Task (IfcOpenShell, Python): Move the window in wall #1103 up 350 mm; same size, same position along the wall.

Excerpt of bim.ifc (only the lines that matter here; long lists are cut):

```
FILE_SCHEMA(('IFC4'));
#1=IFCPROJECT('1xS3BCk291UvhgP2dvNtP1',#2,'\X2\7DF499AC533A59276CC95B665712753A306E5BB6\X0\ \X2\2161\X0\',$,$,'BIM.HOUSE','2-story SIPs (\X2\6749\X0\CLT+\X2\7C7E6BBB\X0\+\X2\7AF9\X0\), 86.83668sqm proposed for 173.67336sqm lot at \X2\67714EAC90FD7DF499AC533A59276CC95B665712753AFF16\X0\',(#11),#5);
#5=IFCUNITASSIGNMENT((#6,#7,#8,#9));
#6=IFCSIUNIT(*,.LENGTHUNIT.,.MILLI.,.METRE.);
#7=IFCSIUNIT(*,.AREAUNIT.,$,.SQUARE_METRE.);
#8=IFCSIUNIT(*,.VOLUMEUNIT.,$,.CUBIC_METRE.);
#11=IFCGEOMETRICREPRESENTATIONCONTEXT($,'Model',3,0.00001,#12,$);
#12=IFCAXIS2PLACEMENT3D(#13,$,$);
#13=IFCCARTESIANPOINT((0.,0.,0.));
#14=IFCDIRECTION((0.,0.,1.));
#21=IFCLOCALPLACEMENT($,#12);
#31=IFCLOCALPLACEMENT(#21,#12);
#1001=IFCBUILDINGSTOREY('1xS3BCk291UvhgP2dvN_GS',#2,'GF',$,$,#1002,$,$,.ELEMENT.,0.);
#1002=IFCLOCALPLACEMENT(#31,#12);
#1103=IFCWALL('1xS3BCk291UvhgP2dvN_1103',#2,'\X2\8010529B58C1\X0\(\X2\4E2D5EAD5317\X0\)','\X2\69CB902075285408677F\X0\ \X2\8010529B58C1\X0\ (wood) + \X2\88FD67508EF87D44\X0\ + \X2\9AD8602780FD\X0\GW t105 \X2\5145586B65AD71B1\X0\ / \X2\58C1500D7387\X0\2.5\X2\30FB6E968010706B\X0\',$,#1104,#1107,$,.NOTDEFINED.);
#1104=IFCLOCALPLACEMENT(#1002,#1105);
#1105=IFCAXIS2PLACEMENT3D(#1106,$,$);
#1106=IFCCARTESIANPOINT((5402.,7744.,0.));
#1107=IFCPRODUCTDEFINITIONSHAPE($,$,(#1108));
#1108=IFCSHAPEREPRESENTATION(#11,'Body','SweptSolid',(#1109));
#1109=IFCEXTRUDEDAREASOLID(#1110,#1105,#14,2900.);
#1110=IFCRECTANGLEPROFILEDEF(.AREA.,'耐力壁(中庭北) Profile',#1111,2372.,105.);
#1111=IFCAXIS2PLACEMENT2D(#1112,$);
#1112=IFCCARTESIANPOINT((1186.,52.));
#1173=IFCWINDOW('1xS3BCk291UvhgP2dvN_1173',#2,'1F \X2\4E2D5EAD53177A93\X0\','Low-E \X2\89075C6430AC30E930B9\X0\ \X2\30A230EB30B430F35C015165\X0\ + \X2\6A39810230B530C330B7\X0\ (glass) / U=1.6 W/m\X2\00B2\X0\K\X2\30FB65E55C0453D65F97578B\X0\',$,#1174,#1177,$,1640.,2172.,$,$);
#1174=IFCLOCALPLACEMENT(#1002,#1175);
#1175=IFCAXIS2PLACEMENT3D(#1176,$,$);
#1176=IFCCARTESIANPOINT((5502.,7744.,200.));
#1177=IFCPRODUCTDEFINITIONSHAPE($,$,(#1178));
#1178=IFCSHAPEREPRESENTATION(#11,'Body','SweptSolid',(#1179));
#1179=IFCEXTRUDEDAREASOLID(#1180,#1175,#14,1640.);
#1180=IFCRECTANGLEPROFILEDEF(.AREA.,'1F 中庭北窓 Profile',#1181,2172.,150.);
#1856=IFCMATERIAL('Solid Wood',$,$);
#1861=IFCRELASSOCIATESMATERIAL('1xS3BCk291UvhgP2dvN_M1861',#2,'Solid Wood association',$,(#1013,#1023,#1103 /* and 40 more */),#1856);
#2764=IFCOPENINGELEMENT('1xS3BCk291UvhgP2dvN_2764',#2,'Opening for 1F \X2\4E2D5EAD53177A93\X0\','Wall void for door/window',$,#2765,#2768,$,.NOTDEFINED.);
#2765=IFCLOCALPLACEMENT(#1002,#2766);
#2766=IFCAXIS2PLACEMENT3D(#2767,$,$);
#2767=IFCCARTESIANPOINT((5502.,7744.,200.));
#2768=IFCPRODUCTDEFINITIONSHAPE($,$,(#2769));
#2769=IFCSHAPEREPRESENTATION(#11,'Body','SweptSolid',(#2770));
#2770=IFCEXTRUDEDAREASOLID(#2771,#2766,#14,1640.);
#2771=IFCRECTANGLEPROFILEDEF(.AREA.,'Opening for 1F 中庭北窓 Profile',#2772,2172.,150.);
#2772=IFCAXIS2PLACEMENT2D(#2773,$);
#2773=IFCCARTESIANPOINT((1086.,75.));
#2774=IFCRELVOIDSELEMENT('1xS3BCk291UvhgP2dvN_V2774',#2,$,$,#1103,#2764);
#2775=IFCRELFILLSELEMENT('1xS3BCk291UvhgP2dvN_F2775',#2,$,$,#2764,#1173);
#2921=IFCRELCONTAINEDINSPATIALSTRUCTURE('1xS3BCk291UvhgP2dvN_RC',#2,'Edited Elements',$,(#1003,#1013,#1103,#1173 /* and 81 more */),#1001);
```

```python
import numpy as np
import ifcopenshell
import ifcopenshell.api.geometry
import ifcopenshell.util.placement
import ifcopenshell.util.unit

model = ifcopenshell.open("bim.ifc")
unit_scale = ifcopenshell.util.unit.calculate_unit_scale(model)

window = model.by_id(1173)
opening = window.FillsVoids[0].RelatingOpeningElement
dz = 350.0

shift = np.array([0.0, 0.0, dz])
# The window is not placed relative to its opening, so move both.
for product in (opening, window):
    matrix = ifcopenshell.util.placement.get_local_placement(product.ObjectPlacement)
    matrix[:3, 3] += shift
    ifcopenshell.api.geometry.edit_object_placement(model, product=product, matrix=matrix, is_si=False)

print(f"moved by {dz * unit_scale:+.3f} m")

model.write("bim_rev.ifc")
```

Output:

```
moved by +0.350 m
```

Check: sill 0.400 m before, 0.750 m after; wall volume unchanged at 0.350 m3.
